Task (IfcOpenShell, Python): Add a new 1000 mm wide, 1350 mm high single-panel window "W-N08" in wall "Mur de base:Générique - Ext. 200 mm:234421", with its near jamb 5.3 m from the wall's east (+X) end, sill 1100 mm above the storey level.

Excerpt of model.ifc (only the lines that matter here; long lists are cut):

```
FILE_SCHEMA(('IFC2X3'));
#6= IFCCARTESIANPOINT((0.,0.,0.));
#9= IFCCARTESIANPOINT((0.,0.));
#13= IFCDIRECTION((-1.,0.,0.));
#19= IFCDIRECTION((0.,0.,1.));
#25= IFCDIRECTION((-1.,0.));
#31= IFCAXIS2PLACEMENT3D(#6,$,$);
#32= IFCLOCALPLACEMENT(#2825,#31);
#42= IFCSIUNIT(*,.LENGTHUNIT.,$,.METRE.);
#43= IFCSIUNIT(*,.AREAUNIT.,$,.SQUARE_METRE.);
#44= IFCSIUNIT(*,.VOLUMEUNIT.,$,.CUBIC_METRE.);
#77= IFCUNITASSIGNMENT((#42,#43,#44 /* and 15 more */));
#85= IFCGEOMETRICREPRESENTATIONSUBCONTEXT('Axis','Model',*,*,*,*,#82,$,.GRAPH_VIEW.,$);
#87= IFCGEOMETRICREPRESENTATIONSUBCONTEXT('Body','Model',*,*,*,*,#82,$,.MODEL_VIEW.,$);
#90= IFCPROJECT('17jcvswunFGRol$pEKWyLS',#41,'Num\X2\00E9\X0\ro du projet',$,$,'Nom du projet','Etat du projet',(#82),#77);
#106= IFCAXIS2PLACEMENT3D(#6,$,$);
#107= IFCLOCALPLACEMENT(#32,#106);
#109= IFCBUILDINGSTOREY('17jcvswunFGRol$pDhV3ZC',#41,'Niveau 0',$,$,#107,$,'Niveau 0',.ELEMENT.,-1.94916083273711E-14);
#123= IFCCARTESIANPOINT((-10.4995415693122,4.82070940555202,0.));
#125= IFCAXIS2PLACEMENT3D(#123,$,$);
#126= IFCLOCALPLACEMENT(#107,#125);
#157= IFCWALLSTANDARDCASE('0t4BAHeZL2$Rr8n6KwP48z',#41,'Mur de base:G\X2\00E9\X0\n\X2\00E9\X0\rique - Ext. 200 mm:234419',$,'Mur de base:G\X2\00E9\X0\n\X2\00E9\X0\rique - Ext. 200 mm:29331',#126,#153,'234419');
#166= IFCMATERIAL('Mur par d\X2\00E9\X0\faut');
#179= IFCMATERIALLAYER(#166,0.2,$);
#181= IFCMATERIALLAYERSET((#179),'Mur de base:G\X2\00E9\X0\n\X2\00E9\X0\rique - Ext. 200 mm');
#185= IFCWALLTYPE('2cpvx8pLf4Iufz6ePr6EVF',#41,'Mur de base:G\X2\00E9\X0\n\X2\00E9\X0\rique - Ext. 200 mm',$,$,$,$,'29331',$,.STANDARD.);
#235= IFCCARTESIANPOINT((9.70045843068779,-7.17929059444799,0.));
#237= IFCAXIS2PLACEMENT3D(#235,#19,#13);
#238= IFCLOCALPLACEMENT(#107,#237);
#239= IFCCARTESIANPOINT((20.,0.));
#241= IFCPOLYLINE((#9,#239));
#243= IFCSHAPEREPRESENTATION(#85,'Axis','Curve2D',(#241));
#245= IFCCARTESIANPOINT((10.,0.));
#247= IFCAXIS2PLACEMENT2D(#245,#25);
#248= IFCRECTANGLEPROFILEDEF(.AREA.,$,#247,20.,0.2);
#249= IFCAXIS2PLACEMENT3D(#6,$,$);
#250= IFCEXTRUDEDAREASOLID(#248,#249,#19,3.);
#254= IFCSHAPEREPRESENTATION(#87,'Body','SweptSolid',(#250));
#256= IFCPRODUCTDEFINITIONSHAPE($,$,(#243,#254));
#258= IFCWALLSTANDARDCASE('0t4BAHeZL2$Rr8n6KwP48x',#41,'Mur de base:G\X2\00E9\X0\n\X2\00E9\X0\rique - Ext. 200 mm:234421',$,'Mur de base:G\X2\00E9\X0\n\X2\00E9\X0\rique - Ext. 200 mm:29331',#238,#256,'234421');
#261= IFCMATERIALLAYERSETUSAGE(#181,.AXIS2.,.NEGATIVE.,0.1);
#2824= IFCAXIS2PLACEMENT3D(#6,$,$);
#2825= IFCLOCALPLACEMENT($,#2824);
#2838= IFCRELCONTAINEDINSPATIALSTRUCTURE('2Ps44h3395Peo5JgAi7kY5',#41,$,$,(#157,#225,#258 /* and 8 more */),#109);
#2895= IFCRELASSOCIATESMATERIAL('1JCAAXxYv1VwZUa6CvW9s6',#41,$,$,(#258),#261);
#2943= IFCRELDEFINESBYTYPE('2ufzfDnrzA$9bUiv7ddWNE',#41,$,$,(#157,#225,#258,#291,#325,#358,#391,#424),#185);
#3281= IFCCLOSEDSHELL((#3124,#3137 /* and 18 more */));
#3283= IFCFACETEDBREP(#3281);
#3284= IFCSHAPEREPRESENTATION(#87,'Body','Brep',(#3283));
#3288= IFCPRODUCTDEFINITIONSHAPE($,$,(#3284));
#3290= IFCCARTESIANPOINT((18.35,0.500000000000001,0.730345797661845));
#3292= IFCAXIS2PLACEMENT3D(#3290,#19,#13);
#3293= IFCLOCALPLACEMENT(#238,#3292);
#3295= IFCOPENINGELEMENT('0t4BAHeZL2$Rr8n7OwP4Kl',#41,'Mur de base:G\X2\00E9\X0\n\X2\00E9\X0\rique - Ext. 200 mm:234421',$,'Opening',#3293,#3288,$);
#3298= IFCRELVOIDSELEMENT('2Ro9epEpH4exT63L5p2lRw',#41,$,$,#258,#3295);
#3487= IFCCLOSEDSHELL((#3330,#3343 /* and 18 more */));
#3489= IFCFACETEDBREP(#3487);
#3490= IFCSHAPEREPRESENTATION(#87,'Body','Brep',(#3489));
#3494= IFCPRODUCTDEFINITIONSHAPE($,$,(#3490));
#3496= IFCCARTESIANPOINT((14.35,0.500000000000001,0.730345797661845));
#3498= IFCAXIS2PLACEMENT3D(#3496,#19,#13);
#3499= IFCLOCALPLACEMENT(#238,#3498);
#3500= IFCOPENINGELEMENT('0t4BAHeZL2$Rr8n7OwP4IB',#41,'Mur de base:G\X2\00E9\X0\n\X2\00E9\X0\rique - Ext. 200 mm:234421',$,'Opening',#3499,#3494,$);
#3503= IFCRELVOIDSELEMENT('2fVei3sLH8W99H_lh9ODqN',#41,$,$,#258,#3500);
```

```python
import numpy as np
import ifcopenshell
import ifcopenshell.api.feature
import ifcopenshell.api.geometry
import ifcopenshell.api.root
import ifcopenshell.api.spatial
import ifcopenshell.api.type
import ifcopenshell.geom
import ifcopenshell.util.element
import ifcopenshell.util.placement
import ifcopenshell.util.representation
import ifcopenshell.util.shape
import ifcopenshell.util.unit

model = ifcopenshell.open("model.ifc")
unit_scale = ifcopenshell.util.unit.calculate_unit_scale(model)
settings = ifcopenshell.geom.settings()


def volume(element):
    """Net volume in cubic metres, openings subtracted."""
    shape = ifcopenshell.geom.create_shape(settings, element)
    return ifcopenshell.util.shape.get_volume(shape.geometry)


wall = model.by_id(258)
storey = ifcopenshell.util.element.get_container(wall, ifc_class="IfcBuildingStorey")
context = ifcopenshell.util.representation.get_context(model, "Model", "Body", "MODEL_VIEW")
before = volume(wall)

width, height, from_end, sill = 1, 1.35, 5.3, 1.1  # metres

# The wall runs along its own X axis, and the end named is its -X end.
wall_shape = ifcopenshell.geom.create_shape(settings, wall)
x, y, z = ifcopenshell.util.shape.get_vertices(wall_shape.geometry).T
start = x.min() + from_end
face, thickness = float(y.min()), float(y.max() - y.min())
wall_matrix = ifcopenshell.util.placement.get_local_placement(wall.ObjectPlacement)
level = ifcopenshell.util.placement.get_local_placement(storey.ObjectPlacement)[2, 3]


def in_wall(x, y):
    """Placement at x, y metres in the wall's axes, at sill height."""
    matrix = wall_matrix.copy()
    matrix[:, 3] = wall_matrix @ np.array([x / unit_scale, y / unit_scale, 0.0, 1.0])
    matrix[2, 3] = level + sill / unit_scale
    return matrix


# Opening: a box that overshoots both wall faces by 50 mm.
opening = ifcopenshell.api.root.create_entity(model, ifc_class="IfcOpeningElement")
box = ifcopenshell.api.geometry.add_wall_representation(
    model, context=context, length=width, height=height, thickness=thickness + 0.1
)
ifcopenshell.api.geometry.assign_representation(model, product=opening, representation=box)
ifcopenshell.api.geometry.edit_object_placement(model, product=opening, matrix=in_wall(start, face - 0.05), is_si=False)
ifcopenshell.api.feature.add_feature(model, feature=opening, element=wall)

window = ifcopenshell.api.root.create_entity(model, ifc_class="IfcWindow", name="W-N08")
window.OverallWidth, window.OverallHeight = width / unit_scale, height / unit_scale
body = ifcopenshell.api.geometry.add_window_representation(
    model,
    context=context,
    overall_width=window.OverallWidth,
    overall_height=window.OverallHeight,
    partition_type="SINGLE_PANEL",
)
ifcopenshell.api.geometry.assign_representation(model, product=window, representation=body)
ifcopenshell.api.spatial.assign_container(model, products=[window], relating_structure=storey)
fills = ifcopenshell.api.feature.add_filling(model, opening=opening, element=window)
fills.OwnerHistory = window.OwnerHistory  # required in IFC2X3

# IFC2X3 keeps the operation on the window style.
style = ifcopenshell.api.root.create_entity(model, ifc_class="IfcWindowStyle", name="W-N08")
style.OperationType, style.ConstructionType = "SINGLE_PANEL", "NOTDEFINED"
style.ParameterTakesPrecedence = style.Sizeable = False
ifcopenshell.api.type.assign_type(model, related_objects=[window], relating_type=style)

# Centre the window in the wall's thickness.
ifcopenshell.api.geometry.edit_object_placement(model, product=window, matrix=in_wall(start, face), is_si=False)
window_shape = ifcopenshell.geom.create_shape(settings, window)
depth = ifcopenshell.util.shape.get_vertices(window_shape.geometry)[:, 1]
offset = face + thickness / 2 - (depth.min() + depth.max()) / 2
ifcopenshell.api.geometry.edit_object_placement(model, product=window, matrix=in_wall(start, offset), is_si=False)

after = volume(wall)

print(f"wall volume {before:.3f} -> {after:.3f} m3")

model.write("model_edited.ifc")
```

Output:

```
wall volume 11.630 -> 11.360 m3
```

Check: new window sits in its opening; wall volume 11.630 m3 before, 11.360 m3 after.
